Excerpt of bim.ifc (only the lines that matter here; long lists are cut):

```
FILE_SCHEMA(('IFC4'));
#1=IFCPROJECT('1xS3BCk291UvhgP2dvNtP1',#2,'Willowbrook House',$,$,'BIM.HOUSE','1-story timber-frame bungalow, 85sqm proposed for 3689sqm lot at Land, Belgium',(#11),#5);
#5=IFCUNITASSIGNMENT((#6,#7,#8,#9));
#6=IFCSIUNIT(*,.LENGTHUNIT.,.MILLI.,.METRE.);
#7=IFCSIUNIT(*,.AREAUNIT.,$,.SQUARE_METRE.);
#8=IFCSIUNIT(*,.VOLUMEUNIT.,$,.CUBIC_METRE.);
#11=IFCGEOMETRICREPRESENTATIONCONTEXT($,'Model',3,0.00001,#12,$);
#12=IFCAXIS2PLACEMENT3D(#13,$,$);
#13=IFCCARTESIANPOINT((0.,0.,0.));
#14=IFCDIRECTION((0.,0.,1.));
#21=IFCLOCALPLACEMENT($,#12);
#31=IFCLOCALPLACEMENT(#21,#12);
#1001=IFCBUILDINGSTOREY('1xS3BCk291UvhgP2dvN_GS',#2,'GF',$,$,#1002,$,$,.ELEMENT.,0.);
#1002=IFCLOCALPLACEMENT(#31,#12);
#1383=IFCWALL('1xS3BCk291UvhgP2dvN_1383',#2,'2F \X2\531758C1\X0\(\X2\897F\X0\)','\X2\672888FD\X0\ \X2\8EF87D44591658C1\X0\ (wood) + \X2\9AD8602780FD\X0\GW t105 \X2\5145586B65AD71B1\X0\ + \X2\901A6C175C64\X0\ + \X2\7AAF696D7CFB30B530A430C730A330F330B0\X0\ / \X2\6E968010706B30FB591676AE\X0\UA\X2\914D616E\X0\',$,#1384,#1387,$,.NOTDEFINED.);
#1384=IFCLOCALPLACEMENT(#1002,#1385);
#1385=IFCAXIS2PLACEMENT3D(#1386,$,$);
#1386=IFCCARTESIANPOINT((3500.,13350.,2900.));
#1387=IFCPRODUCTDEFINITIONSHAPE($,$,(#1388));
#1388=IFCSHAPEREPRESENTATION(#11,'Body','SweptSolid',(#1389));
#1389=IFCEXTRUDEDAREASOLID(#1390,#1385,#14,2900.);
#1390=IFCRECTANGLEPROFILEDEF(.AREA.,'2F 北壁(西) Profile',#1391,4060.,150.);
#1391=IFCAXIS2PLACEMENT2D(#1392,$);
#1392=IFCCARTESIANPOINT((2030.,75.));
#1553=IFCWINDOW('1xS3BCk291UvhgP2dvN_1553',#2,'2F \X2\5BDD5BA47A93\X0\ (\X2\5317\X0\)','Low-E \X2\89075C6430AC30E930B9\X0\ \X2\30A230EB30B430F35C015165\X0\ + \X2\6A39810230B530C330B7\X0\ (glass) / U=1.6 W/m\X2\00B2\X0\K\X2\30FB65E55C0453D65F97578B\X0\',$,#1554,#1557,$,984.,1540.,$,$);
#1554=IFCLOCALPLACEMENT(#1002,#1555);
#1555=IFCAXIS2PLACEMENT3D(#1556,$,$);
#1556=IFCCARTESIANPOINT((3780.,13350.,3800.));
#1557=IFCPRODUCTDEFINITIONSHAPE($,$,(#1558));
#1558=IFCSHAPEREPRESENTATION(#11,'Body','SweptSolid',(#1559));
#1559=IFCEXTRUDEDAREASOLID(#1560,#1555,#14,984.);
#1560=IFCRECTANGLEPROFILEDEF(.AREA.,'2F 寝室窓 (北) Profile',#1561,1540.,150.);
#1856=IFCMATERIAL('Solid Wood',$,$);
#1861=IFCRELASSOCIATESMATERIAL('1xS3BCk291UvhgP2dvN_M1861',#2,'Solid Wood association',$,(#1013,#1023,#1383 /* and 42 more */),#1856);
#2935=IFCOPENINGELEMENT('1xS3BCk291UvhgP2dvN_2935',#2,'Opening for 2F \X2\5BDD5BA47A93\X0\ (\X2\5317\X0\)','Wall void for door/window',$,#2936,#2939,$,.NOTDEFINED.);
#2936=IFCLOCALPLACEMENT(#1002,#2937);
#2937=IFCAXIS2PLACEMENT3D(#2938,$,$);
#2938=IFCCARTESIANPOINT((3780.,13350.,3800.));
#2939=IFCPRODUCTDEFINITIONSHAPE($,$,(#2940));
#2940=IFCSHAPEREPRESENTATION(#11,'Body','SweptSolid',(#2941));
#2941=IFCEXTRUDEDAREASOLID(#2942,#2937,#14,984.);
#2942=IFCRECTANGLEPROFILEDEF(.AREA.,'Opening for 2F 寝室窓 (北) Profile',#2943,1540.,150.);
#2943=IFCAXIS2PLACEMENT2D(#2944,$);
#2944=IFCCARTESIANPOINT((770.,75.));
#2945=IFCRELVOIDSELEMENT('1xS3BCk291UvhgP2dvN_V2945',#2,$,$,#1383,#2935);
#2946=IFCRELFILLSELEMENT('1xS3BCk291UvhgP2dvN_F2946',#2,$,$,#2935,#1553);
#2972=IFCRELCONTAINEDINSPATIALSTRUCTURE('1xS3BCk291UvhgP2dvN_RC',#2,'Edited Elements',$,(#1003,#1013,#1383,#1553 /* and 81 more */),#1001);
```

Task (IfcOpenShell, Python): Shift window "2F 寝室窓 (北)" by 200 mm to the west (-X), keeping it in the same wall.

```python
import ifcopenshell
import ifcopenshell.api.geometry
import ifcopenshell.util.placement

model = ifcopenshell.open("bim.ifc")

window = model.by_id(1553)
opening = window.FillsVoids[0].RelatingOpeningElement
wall = opening.VoidsElements[0].RelatingBuildingElement

wall_matrix = ifcopenshell.util.placement.get_local_placement(wall.ObjectPlacement)
shift = wall_matrix[:3, 0] * -200.0
before = ifcopenshell.util.placement.get_local_placement(window.ObjectPlacement)[:3, 3].copy()

# The window is not placed relative to its opening, so move both.
for product in (opening, window):
    matrix = ifcopenshell.util.placement.get_local_placement(product.ObjectPlacement)
    matrix[:3, 3] += shift
    ifcopenshell.api.geometry.edit_object_placement(model, product=product, matrix=matrix, is_si=False)

after = ifcopenshell.util.placement.get_local_placement(window.ObjectPlacement)[:3, 3]
print("window moved by", (after - before).round(3) + 0.0)

model.write("bim_rev.ifc")
```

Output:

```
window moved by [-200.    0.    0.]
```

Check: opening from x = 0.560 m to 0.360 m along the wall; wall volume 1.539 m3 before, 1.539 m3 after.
